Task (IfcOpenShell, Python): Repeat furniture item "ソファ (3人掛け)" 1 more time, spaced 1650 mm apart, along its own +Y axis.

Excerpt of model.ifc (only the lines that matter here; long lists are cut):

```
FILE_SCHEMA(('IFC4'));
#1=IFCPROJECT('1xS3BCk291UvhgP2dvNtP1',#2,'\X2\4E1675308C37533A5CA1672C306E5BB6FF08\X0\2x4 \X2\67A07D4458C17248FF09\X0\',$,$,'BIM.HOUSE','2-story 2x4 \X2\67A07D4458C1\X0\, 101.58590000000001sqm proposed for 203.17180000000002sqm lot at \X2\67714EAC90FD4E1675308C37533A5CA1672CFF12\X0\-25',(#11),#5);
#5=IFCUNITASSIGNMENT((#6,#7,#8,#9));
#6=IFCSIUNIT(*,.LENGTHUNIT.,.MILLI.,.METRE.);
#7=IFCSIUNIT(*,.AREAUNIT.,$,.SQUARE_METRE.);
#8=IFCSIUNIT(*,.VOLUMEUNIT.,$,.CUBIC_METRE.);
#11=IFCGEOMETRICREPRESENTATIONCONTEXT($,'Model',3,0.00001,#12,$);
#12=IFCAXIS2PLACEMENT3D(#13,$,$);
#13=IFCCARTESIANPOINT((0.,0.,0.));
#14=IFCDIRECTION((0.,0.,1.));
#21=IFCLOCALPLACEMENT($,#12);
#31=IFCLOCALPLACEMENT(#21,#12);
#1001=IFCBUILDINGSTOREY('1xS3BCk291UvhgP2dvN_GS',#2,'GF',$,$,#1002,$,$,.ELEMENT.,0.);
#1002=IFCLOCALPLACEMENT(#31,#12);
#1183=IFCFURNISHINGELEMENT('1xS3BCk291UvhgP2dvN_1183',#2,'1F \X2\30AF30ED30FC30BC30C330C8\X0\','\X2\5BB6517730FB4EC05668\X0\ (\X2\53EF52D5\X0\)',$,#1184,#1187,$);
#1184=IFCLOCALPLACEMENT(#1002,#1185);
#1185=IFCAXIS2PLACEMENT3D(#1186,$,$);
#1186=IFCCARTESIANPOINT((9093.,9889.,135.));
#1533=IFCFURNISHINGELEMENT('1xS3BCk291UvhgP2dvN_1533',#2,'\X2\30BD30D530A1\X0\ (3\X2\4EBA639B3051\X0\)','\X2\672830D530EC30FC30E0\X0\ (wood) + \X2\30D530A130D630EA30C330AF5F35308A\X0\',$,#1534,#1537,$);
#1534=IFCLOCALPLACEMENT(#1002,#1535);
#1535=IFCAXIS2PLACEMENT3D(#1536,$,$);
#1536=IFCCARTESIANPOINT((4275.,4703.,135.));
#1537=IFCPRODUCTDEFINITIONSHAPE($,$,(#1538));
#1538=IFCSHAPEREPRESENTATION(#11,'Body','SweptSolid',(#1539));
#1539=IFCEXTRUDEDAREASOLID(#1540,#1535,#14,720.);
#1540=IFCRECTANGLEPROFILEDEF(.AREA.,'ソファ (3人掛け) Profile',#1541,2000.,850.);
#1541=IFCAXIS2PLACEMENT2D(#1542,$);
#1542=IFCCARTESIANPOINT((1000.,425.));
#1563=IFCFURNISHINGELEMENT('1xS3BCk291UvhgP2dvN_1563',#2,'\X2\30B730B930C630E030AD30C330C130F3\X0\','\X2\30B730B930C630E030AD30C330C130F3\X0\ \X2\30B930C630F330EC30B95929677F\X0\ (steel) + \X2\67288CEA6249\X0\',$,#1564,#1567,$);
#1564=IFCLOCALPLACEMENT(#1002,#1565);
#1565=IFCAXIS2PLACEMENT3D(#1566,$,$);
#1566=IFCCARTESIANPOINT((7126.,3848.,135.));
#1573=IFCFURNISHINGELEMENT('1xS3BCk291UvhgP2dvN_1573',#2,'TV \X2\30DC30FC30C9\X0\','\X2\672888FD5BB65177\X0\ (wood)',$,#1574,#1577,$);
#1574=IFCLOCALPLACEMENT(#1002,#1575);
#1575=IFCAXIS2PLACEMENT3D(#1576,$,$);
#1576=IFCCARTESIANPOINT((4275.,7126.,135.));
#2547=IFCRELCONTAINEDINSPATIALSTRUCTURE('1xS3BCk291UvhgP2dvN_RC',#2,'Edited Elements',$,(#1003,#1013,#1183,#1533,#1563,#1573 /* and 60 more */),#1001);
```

```python
import ifcopenshell
import ifcopenshell.api.geometry
import ifcopenshell.api.root
import ifcopenshell.util.element
import ifcopenshell.util.placement

model = ifcopenshell.open("model.ifc")


def reuse_history(source, copy):
    """copy_class also copies each property set's owner history, people and application; keep the originals."""
    for rel in copy.IsDefinedBy:
        if rel.is_a("IfcRelDefinesByProperties") and (history := rel.RelatingPropertyDefinition.OwnerHistory):
            rel.RelatingPropertyDefinition.OwnerHistory = source.OwnerHistory
            ifcopenshell.util.element.remove_deep2(model, history)


source = model.by_guid("1xS3BCk291UvhgP2dvN_1533")
base = ifcopenshell.util.placement.get_local_placement(source.ObjectPlacement)
step = base[:3, 1] * 1650.0

for i in range(1, 2):
    copy = ifcopenshell.api.root.copy_class(model, product=source)
    copy.Representation = ifcopenshell.util.element.copy_deep(
        model, source.Representation, exclude=["IfcGeometricRepresentationContext", "IfcRepresentationMap"]
    )
    reuse_history(source, copy)
    matrix = base.copy()
    matrix[:3, 3] += i * step
    print("added at", matrix[:3, 3].round(3) + 0.0)
    ifcopenshell.api.geometry.edit_object_placement(model, product=copy, matrix=matrix, is_si=False)

model.write("model_updated.ifc")
```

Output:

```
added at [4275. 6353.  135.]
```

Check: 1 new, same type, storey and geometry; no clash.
